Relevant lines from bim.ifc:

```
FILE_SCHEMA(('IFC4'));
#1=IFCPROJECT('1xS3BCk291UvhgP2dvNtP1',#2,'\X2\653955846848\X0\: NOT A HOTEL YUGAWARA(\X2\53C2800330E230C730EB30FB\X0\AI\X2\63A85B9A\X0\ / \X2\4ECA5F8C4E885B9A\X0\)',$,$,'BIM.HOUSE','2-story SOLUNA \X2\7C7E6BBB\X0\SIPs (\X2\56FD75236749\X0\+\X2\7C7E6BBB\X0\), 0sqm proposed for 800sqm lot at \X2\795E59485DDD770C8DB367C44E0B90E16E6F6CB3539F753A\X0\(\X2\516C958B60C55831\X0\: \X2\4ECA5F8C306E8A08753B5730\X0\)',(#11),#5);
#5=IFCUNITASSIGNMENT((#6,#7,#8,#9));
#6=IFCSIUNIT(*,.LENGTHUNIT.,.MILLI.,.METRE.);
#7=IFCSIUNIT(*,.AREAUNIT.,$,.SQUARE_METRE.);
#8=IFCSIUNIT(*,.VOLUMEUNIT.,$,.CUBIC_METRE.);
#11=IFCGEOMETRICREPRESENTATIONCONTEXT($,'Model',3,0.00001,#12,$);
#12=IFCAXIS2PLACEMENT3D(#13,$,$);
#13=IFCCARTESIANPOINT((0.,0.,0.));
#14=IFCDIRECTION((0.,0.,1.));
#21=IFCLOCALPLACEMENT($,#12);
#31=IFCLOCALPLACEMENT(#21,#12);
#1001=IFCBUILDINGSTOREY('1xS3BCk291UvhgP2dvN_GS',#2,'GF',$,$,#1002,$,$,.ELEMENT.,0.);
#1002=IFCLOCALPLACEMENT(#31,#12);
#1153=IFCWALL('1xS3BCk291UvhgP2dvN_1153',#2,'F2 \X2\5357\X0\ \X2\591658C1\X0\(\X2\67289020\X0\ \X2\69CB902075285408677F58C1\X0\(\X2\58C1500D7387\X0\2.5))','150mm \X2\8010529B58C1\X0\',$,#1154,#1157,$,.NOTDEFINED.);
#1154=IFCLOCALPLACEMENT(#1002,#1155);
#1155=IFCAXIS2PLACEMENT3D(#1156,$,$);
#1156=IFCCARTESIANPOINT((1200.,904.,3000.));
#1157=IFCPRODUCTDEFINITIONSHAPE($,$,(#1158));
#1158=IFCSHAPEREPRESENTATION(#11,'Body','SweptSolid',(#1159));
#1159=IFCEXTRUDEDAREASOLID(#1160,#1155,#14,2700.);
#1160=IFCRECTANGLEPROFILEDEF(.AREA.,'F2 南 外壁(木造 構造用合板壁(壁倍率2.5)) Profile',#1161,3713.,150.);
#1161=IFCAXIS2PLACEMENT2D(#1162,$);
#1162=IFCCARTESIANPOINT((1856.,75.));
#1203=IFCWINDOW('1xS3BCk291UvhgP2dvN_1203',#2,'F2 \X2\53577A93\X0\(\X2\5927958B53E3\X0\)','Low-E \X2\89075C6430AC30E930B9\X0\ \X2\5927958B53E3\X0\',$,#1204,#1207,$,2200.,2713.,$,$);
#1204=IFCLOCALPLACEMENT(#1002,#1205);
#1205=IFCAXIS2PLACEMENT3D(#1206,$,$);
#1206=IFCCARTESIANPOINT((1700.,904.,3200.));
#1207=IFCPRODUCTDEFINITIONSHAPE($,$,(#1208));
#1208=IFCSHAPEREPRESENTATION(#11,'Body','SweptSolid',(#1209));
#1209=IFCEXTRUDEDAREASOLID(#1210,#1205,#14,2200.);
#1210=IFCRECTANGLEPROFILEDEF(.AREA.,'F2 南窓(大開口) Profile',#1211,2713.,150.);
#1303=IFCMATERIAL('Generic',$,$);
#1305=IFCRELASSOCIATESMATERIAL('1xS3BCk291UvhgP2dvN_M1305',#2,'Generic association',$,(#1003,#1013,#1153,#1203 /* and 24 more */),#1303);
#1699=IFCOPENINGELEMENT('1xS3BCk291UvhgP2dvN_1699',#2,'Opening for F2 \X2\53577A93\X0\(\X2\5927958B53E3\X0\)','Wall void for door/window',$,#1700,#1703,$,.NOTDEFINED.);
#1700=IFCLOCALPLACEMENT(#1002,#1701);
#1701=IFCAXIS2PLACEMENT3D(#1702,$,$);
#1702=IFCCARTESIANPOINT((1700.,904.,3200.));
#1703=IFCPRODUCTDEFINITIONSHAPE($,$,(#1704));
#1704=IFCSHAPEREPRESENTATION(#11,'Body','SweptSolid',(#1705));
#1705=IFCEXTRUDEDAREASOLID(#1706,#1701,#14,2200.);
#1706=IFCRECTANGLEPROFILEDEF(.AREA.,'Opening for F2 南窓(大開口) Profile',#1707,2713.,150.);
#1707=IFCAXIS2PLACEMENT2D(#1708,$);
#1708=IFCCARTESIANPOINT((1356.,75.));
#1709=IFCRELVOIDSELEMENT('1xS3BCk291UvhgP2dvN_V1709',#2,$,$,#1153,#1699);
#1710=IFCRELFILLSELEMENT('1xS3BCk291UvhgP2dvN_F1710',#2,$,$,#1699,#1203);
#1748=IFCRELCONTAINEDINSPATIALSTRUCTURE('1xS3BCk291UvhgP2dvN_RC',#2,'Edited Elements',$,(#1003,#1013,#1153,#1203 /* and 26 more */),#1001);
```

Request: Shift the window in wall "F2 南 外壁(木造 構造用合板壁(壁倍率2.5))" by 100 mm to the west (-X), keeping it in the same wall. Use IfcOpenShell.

```python
import ifcopenshell
import ifcopenshell.api.geometry
import ifcopenshell.util.placement
import ifcopenshell.util.unit

model = ifcopenshell.open("bim.ifc")
unit_scale = ifcopenshell.util.unit.calculate_unit_scale(model)

window = model.by_guid("1xS3BCk291UvhgP2dvN_1203")
opening = window.FillsVoids[0].RelatingOpeningElement
wall = opening.VoidsElements[0].RelatingBuildingElement

wall_matrix = ifcopenshell.util.placement.get_local_placement(wall.ObjectPlacement)
shift = wall_matrix[:3, 0] * -0.1 / unit_scale
before = ifcopenshell.util.placement.get_local_placement(window.ObjectPlacement)[:3, 3].copy()

# The window is not placed relative to its opening, so move both.
for product in (opening, window):
    matrix = ifcopenshell.util.placement.get_local_placement(product.ObjectPlacement)
    matrix[:3, 3] += shift
    ifcopenshell.api.geometry.edit_object_placement(model, product=product, matrix=matrix, is_si=False)

after = ifcopenshell.util.placement.get_local_placement(window.ObjectPlacement)[:3, 3]
print("window moved by", (after - before).round(3) + 0.0)

model.write("bim_updated.ifc")
```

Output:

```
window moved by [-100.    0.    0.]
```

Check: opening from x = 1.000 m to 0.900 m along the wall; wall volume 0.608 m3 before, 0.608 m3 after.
